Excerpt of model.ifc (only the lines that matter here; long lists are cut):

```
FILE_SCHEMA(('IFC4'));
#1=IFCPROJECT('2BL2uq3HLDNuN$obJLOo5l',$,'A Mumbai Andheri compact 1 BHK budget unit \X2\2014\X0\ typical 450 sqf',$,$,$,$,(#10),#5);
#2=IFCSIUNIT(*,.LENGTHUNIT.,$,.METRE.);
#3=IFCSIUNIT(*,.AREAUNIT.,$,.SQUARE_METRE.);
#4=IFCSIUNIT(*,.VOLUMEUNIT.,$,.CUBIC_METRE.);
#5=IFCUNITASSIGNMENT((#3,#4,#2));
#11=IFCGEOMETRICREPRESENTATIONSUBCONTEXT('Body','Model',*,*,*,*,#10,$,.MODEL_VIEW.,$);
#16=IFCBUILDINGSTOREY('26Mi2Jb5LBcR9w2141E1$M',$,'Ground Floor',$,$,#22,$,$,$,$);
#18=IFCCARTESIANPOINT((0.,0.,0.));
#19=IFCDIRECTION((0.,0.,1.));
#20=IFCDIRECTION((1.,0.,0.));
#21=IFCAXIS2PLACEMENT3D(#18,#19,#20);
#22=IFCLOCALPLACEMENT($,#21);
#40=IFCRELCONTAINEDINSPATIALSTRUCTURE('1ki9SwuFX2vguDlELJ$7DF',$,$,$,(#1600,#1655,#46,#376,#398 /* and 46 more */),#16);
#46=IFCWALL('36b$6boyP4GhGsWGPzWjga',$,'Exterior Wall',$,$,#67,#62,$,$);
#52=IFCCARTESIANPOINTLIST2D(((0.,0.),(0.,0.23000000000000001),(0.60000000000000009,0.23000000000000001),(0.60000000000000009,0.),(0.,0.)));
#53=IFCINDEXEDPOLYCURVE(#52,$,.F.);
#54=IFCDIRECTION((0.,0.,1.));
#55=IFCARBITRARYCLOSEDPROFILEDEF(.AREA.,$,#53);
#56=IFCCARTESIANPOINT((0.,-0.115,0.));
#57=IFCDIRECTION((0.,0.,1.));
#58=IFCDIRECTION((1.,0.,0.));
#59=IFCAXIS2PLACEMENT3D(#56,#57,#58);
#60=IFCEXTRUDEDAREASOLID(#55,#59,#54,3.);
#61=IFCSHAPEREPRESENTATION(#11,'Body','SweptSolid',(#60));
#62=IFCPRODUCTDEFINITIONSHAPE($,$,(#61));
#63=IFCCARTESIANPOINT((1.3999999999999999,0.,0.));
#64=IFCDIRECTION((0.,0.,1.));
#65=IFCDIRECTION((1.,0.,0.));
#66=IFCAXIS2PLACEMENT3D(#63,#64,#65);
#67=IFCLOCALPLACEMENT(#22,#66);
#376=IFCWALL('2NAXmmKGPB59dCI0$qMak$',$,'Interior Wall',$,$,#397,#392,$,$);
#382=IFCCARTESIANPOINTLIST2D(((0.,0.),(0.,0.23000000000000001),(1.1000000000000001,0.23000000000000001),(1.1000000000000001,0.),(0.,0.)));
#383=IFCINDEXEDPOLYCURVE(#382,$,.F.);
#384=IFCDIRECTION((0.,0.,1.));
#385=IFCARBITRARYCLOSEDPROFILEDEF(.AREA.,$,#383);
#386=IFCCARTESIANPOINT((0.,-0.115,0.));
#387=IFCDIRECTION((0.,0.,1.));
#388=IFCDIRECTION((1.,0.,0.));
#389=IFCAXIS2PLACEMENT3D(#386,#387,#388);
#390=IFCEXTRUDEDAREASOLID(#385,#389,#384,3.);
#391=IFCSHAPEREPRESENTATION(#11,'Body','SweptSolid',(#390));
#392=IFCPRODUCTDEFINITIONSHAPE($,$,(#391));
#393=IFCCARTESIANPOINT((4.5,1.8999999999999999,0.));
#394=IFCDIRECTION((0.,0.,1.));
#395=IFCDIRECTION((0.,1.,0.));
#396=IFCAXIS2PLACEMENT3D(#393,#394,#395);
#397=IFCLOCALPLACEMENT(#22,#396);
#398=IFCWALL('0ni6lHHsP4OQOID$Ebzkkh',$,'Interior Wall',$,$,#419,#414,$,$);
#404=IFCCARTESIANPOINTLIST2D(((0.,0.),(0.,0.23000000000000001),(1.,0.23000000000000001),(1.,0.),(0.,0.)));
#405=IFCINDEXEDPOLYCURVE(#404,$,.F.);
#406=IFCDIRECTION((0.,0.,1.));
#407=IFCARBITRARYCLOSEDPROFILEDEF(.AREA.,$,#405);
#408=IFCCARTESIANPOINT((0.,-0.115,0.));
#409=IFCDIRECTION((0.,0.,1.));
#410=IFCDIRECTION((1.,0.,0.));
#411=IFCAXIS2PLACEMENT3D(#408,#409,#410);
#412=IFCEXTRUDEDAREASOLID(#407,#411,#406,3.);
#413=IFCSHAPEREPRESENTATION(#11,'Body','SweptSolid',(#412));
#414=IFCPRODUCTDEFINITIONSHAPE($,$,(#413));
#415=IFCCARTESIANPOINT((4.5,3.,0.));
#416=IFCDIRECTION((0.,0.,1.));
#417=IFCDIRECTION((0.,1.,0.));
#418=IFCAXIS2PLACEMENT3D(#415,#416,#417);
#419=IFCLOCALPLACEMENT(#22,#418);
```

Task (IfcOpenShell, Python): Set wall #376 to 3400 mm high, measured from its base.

```python
import ifcopenshell
import ifcopenshell.geom
import ifcopenshell.util.representation
import ifcopenshell.util.shape
import ifcopenshell.util.unit

model = ifcopenshell.open("model.ifc")
unit_scale = ifcopenshell.util.unit.calculate_unit_scale(model)
settings = ifcopenshell.geom.settings()


def volume(element):
    """Net volume in cubic metres, openings subtracted."""
    shape = ifcopenshell.geom.create_shape(settings, element)
    return ifcopenshell.util.shape.get_volume(shape.geometry)


wall = model.by_guid("2NAXmmKGPB59dCI0$qMak$")
before = volume(wall)

body = ifcopenshell.util.representation.get_representation(wall, "Model", "Body")
solid = body.Items[0]
old_height = solid.Depth
solid.Depth = 3.4 / unit_scale
after = volume(wall)

print(f"height {old_height:g} -> {solid.Depth:g}, volume {before:.3f} -> {after:.3f} m3")

model.write("model_v2.ifc")
```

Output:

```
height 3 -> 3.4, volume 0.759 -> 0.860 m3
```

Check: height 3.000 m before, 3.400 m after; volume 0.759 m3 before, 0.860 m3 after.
